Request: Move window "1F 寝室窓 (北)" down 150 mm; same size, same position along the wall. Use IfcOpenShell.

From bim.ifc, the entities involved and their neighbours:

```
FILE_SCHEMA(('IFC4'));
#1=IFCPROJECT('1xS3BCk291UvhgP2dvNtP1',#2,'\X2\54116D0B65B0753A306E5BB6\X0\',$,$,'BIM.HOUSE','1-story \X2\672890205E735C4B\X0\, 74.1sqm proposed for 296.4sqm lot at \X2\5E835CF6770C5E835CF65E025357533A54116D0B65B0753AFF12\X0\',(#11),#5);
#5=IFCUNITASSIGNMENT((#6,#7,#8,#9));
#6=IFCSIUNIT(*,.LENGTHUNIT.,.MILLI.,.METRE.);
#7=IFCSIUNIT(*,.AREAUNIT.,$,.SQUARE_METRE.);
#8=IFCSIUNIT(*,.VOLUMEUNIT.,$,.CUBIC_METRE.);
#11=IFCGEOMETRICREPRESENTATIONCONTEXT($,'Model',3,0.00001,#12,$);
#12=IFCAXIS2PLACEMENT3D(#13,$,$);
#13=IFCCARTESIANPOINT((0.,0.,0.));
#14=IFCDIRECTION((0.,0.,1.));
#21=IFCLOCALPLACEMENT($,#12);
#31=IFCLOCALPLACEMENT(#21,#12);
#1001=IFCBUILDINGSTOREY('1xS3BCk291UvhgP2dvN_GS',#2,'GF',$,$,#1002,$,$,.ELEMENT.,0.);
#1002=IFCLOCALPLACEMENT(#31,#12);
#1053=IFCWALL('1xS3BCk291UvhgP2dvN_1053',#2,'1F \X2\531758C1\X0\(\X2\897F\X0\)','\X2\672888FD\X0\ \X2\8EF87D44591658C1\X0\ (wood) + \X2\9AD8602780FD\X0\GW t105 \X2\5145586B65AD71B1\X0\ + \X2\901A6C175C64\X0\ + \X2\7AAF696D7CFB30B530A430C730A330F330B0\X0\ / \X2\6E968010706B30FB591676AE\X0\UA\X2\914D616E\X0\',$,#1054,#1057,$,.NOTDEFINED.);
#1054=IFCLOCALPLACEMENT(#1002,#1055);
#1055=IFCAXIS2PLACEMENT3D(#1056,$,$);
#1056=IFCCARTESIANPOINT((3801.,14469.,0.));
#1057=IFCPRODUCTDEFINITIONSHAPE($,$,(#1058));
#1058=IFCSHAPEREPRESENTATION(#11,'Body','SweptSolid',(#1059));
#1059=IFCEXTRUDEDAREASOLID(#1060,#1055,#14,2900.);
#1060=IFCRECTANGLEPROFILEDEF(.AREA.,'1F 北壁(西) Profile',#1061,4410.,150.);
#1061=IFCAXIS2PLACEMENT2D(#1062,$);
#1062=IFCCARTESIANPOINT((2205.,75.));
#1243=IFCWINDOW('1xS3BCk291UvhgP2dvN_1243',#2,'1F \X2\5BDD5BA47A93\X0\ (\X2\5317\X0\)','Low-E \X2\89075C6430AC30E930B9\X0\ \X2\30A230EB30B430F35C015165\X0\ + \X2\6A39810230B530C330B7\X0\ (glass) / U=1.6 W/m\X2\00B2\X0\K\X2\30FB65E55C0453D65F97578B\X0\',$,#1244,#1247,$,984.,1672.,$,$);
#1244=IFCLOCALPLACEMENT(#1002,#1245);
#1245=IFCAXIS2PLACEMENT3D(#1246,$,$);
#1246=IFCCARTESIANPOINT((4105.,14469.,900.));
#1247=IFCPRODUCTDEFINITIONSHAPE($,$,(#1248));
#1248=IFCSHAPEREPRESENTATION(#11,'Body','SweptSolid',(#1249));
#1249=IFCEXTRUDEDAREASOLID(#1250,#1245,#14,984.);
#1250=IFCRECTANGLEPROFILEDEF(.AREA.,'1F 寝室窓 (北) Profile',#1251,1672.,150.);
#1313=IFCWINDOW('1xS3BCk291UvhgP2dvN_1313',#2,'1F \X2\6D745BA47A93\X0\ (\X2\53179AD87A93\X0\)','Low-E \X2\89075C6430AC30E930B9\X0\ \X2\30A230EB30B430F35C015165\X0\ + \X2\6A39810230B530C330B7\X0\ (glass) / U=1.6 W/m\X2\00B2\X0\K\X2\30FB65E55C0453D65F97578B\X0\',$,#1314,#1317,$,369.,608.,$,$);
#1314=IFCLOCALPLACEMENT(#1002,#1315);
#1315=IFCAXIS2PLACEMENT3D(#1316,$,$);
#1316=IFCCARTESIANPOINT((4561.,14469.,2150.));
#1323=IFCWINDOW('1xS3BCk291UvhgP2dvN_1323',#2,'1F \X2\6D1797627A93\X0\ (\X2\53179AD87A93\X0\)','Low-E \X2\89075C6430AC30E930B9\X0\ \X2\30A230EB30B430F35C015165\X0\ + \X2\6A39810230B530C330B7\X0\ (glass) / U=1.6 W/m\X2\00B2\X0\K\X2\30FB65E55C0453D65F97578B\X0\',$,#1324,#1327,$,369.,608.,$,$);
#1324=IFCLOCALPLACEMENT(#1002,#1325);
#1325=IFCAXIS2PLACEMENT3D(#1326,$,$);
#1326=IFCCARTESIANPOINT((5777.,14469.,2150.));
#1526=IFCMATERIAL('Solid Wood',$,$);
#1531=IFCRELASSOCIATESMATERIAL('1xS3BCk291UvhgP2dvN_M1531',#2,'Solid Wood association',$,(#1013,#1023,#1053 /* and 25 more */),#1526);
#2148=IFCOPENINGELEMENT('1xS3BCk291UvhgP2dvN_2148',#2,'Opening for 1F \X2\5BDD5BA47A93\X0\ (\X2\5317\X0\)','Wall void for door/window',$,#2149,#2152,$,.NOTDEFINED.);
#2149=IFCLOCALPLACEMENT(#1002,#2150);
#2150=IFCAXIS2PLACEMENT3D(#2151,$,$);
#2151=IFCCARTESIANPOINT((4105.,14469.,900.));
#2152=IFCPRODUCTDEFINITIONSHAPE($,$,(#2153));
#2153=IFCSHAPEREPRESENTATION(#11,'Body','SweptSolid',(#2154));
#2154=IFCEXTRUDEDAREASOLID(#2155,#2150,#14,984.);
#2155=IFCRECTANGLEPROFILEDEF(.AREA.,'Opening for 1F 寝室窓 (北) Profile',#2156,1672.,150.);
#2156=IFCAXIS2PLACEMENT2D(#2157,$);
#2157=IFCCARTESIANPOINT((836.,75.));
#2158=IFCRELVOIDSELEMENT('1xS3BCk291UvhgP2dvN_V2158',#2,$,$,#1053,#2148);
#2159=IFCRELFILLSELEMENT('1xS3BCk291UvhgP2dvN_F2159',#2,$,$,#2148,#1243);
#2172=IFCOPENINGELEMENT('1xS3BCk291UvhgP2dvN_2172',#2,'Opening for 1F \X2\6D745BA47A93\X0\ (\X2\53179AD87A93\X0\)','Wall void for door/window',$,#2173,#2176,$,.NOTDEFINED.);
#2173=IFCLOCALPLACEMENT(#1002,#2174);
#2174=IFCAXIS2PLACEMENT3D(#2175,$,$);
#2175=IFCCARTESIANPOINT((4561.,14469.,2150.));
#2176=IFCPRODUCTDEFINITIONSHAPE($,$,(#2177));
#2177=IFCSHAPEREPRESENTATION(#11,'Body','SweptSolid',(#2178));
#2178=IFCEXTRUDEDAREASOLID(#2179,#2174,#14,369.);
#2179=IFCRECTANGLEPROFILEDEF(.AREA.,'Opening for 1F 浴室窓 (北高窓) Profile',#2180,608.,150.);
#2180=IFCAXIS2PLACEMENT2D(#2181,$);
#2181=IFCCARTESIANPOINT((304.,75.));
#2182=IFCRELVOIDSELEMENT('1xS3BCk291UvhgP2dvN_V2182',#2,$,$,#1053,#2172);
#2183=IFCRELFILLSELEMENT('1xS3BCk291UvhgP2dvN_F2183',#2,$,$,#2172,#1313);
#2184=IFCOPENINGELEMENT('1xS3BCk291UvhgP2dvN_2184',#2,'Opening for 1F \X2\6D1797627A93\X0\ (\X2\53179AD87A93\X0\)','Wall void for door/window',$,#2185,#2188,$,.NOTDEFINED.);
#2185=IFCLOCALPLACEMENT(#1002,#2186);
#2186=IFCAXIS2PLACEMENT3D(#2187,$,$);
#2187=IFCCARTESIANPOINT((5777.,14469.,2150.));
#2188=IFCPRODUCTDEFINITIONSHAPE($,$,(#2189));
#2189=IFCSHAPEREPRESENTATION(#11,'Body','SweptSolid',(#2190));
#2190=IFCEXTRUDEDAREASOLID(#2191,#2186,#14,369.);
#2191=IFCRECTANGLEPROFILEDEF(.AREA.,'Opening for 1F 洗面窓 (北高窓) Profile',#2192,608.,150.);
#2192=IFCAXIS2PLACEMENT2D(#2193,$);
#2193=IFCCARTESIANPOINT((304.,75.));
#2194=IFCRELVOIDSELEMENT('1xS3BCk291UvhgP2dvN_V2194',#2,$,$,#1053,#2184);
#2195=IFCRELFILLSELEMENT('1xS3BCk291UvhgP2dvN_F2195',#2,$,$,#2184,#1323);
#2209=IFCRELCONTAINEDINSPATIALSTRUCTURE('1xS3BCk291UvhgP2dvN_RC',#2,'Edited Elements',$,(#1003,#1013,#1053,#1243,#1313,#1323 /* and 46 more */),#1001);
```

```python
import numpy as np
import ifcopenshell
import ifcopenshell.api.geometry
import ifcopenshell.util.placement
import ifcopenshell.util.unit

model = ifcopenshell.open("bim.ifc")
unit_scale = ifcopenshell.util.unit.calculate_unit_scale(model)

window = model.by_guid("1xS3BCk291UvhgP2dvN_1243")
opening = window.FillsVoids[0].RelatingOpeningElement
dz = -0.15 / unit_scale

shift = np.array([0.0, 0.0, dz])
# The window is not placed relative to its opening, so move both.
for product in (opening, window):
    matrix = ifcopenshell.util.placement.get_local_placement(product.ObjectPlacement)
    matrix[:3, 3] += shift
    ifcopenshell.api.geometry.edit_object_placement(model, product=product, matrix=matrix, is_si=False)

print(f"moved by {dz * unit_scale:+.3f} m")

model.write("bim_updated.ifc")
```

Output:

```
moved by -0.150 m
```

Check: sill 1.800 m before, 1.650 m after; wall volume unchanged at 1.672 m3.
